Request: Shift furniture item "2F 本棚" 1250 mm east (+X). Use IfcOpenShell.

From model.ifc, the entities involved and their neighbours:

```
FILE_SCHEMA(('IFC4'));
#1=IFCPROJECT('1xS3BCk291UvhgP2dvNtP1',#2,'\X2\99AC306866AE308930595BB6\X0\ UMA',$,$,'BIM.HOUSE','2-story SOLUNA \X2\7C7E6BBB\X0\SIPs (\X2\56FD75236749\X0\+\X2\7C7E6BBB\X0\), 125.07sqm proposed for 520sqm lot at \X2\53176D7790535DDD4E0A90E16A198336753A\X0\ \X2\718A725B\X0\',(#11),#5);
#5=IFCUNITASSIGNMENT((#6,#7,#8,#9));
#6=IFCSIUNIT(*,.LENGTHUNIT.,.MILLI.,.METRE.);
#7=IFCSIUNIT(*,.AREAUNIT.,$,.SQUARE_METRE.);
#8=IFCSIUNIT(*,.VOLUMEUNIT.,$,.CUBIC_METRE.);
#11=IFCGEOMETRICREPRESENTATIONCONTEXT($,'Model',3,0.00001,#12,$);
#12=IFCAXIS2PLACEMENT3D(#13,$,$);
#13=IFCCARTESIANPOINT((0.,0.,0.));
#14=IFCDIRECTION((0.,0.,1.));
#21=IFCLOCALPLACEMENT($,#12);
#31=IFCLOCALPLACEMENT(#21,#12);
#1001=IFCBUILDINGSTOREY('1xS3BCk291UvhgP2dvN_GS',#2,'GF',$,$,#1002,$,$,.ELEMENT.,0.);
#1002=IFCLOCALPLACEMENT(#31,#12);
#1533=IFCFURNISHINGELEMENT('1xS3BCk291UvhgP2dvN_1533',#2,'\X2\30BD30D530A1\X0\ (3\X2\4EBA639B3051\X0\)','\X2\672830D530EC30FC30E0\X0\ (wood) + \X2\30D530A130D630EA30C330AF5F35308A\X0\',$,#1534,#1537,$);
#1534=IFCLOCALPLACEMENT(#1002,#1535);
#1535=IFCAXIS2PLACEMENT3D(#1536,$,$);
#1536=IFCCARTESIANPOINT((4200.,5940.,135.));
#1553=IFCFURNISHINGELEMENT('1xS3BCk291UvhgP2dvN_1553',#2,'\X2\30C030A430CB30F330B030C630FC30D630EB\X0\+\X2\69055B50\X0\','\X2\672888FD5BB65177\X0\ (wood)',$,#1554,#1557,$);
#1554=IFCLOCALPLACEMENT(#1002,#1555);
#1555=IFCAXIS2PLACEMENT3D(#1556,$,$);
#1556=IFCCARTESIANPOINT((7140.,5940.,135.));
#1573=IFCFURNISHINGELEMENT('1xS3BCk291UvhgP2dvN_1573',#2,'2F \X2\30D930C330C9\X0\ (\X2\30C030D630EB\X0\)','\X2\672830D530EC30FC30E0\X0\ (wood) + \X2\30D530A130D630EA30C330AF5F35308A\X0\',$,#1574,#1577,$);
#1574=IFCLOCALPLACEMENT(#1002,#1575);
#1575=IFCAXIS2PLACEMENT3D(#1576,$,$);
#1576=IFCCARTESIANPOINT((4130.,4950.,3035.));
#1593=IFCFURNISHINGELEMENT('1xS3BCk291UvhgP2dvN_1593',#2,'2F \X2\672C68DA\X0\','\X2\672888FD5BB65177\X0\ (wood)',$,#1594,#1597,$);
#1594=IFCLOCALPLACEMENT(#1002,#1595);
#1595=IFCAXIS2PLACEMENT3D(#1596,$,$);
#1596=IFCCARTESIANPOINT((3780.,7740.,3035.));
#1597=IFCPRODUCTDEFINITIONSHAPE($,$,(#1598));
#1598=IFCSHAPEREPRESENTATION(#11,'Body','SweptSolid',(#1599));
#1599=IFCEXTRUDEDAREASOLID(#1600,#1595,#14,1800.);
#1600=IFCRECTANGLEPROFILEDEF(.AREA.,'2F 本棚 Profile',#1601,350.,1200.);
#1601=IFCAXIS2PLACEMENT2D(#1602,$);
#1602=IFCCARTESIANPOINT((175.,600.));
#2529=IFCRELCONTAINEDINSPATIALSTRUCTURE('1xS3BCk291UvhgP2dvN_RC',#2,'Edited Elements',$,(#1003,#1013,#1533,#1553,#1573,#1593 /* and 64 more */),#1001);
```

```python
import ifcopenshell
import ifcopenshell.api.geometry
import ifcopenshell.util.placement
import ifcopenshell.util.unit

model = ifcopenshell.open("model.ifc")
unit_scale = ifcopenshell.util.unit.calculate_unit_scale(model)

item = model.by_guid("1xS3BCk291UvhgP2dvN_1593")
matrix = ifcopenshell.util.placement.get_local_placement(item.ObjectPlacement)
matrix[0, 3] += 1.25 / unit_scale
ifcopenshell.api.geometry.edit_object_placement(model, product=item, matrix=matrix, is_si=False)

print(ifcopenshell.util.placement.get_local_placement(item.ObjectPlacement).round(3) + 0.0)

model.write("model_updated.ifc")
```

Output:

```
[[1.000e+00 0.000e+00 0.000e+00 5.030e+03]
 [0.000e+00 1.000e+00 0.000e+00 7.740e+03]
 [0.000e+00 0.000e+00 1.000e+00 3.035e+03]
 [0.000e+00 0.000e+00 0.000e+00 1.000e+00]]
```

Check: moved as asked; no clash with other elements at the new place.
